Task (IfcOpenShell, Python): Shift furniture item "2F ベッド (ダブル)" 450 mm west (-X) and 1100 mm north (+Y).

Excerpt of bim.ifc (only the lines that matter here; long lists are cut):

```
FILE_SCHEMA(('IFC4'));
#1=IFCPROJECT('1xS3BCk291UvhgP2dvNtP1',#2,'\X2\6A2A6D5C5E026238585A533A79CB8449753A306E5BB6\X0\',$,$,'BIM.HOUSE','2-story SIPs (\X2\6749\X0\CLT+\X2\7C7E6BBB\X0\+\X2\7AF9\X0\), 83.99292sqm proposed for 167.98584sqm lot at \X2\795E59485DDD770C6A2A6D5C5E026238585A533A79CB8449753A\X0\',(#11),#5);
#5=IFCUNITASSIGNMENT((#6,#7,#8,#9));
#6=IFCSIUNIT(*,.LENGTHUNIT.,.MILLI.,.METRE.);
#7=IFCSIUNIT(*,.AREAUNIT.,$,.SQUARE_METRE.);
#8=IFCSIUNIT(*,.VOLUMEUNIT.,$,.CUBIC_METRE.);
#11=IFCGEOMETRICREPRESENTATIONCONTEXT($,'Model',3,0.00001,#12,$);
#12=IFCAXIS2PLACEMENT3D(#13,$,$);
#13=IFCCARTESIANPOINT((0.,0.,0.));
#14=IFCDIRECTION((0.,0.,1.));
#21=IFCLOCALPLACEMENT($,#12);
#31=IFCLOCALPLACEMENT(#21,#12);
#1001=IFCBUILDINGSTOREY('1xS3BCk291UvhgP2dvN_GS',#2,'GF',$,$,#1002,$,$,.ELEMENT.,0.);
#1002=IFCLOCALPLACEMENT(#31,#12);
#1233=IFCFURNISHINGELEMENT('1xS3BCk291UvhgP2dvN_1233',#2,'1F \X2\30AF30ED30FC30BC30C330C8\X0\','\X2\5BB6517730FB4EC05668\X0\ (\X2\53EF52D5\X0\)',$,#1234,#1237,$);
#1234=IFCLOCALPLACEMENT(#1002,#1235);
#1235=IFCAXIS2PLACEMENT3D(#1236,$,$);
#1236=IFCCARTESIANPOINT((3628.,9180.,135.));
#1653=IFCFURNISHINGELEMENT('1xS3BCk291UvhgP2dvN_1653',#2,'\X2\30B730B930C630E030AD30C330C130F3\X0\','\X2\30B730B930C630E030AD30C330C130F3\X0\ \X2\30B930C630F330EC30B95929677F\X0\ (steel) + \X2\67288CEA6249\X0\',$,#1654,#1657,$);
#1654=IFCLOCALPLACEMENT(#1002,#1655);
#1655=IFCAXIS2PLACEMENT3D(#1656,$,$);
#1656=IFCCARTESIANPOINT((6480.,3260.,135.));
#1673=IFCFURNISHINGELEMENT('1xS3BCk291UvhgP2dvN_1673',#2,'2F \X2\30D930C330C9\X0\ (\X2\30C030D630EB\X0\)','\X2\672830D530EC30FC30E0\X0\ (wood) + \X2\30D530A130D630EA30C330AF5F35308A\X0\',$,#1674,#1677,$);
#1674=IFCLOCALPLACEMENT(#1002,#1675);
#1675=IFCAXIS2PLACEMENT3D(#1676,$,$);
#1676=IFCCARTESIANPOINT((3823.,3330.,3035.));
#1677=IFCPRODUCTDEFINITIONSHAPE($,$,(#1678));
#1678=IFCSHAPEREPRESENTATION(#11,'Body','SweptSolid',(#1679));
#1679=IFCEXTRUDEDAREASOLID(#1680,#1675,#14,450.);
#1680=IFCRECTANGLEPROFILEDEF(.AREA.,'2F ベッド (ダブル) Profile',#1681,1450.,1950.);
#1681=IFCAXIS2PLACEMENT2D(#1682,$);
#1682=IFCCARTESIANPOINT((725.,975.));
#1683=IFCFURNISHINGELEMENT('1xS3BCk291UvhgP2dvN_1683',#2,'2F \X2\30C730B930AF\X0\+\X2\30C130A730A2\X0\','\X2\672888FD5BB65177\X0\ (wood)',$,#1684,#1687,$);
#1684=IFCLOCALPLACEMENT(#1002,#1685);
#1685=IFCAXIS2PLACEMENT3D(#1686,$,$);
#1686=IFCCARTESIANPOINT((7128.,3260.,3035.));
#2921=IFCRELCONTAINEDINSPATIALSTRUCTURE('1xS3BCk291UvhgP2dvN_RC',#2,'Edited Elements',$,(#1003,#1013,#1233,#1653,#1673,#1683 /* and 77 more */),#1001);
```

```python
import ifcopenshell
import ifcopenshell.api.geometry
import ifcopenshell.util.placement
import ifcopenshell.util.unit

model = ifcopenshell.open("bim.ifc")
unit_scale = ifcopenshell.util.unit.calculate_unit_scale(model)

item = model.by_guid("1xS3BCk291UvhgP2dvN_1673")
matrix = ifcopenshell.util.placement.get_local_placement(item.ObjectPlacement)
matrix[0, 3] -= 0.45 / unit_scale
matrix[1, 3] += 1.1 / unit_scale
ifcopenshell.api.geometry.edit_object_placement(model, product=item, matrix=matrix, is_si=False)

print(ifcopenshell.util.placement.get_local_placement(item.ObjectPlacement).round(3) + 0.0)

model.write("bim-out.ifc")
```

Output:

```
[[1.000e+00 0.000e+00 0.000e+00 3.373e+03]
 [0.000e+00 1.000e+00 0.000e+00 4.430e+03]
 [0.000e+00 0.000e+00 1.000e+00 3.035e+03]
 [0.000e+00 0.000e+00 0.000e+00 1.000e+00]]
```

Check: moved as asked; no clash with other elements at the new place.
